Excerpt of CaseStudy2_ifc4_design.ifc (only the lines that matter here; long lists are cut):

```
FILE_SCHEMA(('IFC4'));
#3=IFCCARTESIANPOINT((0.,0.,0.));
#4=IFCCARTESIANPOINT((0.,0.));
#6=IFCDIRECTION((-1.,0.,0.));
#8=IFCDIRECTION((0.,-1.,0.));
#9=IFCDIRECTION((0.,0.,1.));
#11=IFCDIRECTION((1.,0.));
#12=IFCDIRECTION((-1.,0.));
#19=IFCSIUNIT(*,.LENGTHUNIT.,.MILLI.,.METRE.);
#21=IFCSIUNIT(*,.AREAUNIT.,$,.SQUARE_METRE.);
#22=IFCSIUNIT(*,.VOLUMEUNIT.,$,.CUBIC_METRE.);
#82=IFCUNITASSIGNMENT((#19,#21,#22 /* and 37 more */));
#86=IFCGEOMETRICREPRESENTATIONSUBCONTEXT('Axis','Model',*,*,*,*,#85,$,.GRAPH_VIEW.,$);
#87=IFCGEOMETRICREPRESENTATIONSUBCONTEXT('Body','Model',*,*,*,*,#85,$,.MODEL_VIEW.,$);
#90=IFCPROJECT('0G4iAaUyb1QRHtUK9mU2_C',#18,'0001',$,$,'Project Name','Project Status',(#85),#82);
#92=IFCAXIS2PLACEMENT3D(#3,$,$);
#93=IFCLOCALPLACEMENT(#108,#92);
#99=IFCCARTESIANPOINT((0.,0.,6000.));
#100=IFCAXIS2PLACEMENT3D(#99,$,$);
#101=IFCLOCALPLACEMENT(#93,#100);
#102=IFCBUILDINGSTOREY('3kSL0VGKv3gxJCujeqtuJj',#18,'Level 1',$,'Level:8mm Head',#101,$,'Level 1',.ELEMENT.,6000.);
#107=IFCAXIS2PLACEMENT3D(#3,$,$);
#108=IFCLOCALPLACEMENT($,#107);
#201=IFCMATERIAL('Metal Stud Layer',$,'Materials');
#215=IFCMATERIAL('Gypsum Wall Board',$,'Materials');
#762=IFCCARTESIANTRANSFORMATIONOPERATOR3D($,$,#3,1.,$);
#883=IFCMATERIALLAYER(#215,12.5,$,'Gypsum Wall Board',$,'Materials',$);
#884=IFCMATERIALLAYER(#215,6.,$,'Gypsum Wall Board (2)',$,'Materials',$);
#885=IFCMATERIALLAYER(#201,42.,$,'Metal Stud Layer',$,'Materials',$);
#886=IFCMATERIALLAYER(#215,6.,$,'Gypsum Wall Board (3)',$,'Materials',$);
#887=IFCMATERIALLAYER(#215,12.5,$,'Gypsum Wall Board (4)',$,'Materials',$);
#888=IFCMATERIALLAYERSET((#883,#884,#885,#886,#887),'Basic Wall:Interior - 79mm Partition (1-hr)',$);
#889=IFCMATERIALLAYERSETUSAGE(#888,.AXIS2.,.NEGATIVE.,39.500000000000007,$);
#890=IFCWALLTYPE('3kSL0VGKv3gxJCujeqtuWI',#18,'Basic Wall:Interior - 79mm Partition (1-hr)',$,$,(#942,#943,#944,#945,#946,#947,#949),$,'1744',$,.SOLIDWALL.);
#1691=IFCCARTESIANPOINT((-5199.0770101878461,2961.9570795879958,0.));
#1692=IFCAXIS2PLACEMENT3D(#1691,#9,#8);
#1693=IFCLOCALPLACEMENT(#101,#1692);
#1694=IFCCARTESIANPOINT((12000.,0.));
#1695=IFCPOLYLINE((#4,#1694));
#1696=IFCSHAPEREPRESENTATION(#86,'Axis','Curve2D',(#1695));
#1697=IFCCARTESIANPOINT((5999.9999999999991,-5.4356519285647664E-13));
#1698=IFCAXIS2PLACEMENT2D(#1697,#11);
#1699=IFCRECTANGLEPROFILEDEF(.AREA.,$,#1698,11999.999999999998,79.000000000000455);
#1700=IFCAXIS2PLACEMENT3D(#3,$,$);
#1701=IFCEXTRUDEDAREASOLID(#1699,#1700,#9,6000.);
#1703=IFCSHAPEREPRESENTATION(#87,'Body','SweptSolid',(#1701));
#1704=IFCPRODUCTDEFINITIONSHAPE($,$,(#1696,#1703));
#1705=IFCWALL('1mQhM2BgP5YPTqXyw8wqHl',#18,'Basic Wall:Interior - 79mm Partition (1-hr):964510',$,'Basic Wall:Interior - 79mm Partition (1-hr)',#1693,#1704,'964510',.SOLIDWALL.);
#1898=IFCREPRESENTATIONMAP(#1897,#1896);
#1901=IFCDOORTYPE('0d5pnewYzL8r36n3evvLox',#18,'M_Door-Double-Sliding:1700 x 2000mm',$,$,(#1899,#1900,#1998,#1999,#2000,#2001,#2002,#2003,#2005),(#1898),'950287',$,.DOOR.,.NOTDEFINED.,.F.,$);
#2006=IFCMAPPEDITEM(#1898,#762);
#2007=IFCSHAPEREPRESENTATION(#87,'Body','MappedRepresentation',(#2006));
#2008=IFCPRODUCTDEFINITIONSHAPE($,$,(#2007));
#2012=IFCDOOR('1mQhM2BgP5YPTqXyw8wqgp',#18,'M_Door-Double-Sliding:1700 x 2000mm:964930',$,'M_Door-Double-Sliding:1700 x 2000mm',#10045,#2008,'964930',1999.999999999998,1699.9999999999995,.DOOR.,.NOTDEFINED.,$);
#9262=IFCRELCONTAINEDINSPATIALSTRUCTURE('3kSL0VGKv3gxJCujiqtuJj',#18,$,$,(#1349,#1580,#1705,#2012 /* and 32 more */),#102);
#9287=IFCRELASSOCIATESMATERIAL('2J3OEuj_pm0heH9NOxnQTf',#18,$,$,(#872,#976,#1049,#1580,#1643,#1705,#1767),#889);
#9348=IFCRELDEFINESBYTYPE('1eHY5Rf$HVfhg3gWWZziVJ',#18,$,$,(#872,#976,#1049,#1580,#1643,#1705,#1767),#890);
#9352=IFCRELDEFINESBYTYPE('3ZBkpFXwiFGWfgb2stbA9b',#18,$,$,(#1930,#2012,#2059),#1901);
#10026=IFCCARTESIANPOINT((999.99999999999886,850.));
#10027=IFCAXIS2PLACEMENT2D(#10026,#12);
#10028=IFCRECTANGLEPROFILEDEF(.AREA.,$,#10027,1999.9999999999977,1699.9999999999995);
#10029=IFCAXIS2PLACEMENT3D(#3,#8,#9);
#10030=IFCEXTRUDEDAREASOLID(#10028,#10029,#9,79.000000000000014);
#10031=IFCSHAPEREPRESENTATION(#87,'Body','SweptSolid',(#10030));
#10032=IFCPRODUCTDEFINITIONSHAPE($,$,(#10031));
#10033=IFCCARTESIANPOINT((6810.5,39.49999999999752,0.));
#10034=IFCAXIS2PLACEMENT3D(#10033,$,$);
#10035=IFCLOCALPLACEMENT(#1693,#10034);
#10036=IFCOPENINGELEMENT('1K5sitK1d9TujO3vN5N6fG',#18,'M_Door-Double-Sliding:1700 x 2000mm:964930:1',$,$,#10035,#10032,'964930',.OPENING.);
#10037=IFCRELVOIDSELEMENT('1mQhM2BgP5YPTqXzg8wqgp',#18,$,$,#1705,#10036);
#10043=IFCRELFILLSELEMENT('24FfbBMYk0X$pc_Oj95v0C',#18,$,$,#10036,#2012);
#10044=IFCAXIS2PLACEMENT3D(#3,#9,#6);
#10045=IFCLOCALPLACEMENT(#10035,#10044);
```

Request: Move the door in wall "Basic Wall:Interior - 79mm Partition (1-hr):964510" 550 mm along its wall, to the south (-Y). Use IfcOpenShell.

```python
import ifcopenshell
import ifcopenshell.api.geometry
import ifcopenshell.util.placement
import ifcopenshell.util.unit

model = ifcopenshell.open("CaseStudy2_ifc4_design.ifc")
unit_scale = ifcopenshell.util.unit.calculate_unit_scale(model)

door = model.by_guid("1mQhM2BgP5YPTqXyw8wqgp")
opening = door.FillsVoids[0].RelatingOpeningElement
wall = opening.VoidsElements[0].RelatingBuildingElement

wall_matrix = ifcopenshell.util.placement.get_local_placement(wall.ObjectPlacement)
shift = wall_matrix[:3, 0] * 0.55 / unit_scale
before = ifcopenshell.util.placement.get_local_placement(door.ObjectPlacement)[:3, 3].copy()

# The door is placed relative to its opening, so it follows when the opening moves.
matrix = ifcopenshell.util.placement.get_local_placement(opening.ObjectPlacement)
matrix[:3, 3] += shift
ifcopenshell.api.geometry.edit_object_placement(
    model, product=opening, matrix=matrix, is_si=False, should_transform_children=True
)

after = ifcopenshell.util.placement.get_local_placement(door.ObjectPlacement)[:3, 3]
print("door moved by", (after - before).round(3) + 0.0)

model.write("CaseStudy2_ifc4_design-out.ifc")
```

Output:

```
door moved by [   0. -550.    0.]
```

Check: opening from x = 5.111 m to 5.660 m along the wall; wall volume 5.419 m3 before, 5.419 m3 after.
